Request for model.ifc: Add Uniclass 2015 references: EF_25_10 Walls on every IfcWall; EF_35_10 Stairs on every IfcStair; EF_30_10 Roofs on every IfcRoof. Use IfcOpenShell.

First a look at what the model holds.

```python
import ifcopenshell

model = ifcopenshell.open("model.ifc")
print(model.schema)
print("classifications:", [c.Name for c in model.by_type("IfcClassification")])
for ifc_class in ("IfcDoor", "IfcRoof", "IfcStair", "IfcWall", "IfcWindow"):
    print(ifc_class, len(model.by_type(ifc_class)))
```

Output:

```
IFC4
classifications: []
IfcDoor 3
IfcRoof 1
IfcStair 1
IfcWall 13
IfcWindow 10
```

```python
import ifcopenshell
import ifcopenshell.api.classification

model = ifcopenshell.open("model.ifc")

system = ifcopenshell.api.classification.add_classification(model, classification="Uniclass 2015")

codes = {
    "IfcWall": ("EF_25_10", "Walls"),
    "IfcStair": ("EF_35_10", "Stairs"),
    "IfcRoof": ("EF_30_10", "Roofs"),
}
for ifc_class, (code, name) in codes.items():
    products = model.by_type(ifc_class)
    ifcopenshell.api.classification.add_reference(
        model, products=products, classification=system, identification=code, name=name
    )
    print(code, len(products))

model.write("model_edited.ifc")
```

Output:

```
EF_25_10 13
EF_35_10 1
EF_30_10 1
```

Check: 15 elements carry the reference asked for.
